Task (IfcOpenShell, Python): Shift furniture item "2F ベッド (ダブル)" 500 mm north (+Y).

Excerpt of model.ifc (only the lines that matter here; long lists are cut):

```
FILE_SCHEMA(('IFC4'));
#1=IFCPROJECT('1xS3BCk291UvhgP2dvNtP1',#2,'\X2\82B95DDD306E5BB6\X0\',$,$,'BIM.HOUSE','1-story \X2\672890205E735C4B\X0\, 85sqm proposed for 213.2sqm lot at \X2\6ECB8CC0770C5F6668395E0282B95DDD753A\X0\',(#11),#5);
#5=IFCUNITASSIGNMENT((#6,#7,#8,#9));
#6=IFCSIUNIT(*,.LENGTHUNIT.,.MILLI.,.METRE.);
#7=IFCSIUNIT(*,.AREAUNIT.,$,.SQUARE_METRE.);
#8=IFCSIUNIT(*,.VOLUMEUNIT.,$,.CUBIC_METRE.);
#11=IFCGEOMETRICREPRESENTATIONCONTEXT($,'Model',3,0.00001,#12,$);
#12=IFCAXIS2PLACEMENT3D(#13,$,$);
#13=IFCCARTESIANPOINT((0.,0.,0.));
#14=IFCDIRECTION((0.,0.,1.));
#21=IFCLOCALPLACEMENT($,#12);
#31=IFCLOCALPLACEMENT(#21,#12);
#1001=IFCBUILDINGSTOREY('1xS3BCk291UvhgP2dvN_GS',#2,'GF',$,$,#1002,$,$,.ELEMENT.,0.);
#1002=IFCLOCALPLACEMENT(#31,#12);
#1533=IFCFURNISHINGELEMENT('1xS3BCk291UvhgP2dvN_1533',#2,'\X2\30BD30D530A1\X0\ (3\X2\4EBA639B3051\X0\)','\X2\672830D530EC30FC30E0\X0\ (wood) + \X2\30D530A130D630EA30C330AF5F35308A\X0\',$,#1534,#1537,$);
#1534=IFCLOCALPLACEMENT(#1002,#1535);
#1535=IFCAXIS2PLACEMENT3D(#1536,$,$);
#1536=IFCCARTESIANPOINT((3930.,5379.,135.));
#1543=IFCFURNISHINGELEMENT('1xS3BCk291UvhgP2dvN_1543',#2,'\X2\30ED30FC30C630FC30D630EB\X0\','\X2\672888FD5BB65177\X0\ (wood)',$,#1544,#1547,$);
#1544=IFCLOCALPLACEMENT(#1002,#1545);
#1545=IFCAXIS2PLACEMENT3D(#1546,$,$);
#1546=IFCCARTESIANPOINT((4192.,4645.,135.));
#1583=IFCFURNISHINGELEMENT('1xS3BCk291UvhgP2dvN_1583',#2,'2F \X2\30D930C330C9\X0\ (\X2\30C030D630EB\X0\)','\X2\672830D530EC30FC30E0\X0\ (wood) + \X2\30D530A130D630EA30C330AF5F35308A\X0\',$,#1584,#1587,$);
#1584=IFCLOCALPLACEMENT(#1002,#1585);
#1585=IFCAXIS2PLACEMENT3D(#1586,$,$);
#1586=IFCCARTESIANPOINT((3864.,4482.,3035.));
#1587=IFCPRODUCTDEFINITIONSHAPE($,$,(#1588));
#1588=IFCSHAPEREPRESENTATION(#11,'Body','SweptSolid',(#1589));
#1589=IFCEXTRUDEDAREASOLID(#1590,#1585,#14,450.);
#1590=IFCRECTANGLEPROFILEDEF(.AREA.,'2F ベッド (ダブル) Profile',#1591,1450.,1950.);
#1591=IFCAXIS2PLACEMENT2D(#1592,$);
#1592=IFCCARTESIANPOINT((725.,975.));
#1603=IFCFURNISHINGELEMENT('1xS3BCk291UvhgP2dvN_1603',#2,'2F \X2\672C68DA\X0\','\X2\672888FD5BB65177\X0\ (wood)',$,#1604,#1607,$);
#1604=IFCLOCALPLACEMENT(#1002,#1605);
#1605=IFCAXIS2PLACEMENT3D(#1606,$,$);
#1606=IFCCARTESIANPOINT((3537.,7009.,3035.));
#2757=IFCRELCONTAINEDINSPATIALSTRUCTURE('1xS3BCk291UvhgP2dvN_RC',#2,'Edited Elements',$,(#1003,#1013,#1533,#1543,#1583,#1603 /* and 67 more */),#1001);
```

```python
import ifcopenshell
import ifcopenshell.api.geometry
import ifcopenshell.util.placement
import ifcopenshell.util.unit

model = ifcopenshell.open("model.ifc")
unit_scale = ifcopenshell.util.unit.calculate_unit_scale(model)

item = model.by_guid("1xS3BCk291UvhgP2dvN_1583")
matrix = ifcopenshell.util.placement.get_local_placement(item.ObjectPlacement)
matrix[1, 3] += 0.5 / unit_scale
ifcopenshell.api.geometry.edit_object_placement(model, product=item, matrix=matrix, is_si=False)

print(ifcopenshell.util.placement.get_local_placement(item.ObjectPlacement).round(3) + 0.0)

model.write("model-out.ifc")
```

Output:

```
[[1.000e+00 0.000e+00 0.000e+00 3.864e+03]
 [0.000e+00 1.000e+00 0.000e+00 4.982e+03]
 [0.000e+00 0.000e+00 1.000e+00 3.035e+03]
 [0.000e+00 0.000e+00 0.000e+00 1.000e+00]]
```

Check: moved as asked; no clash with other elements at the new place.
